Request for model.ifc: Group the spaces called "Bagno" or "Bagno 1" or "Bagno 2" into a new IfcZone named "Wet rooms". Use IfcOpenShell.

First a look at what the model holds.

```python
import ifcopenshell

model = ifcopenshell.open("model.ifc")
print(model.schema)
seen = {}
for space in model.by_type("IfcSpace"):
    seen[space.LongName] = seen.get(space.LongName, 0) + 1
for name, count in sorted(seen.items(), key=str):
    print(count, "x", name)
print("zones:", [z.Name for z in model.by_type("IfcZone")][:20])
```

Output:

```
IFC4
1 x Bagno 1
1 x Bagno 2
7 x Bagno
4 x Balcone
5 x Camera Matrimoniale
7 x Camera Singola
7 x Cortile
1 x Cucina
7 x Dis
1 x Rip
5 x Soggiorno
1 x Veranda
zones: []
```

```python
import ifcopenshell
import ifcopenshell.api.group
import ifcopenshell.api.root

model = ifcopenshell.open("model.ifc")

names = {"Bagno", "Bagno 1", "Bagno 2"}
spaces = [s for s in model.by_type("IfcSpace") if s.LongName in names]

zone = ifcopenshell.api.root.create_entity(model, ifc_class="IfcZone", name="Wet rooms")
ifcopenshell.api.group.assign_group(model, products=spaces, group=zone)
print(len(spaces), "spaces in", zone.Name)

model.write("model_rev.ifc")
```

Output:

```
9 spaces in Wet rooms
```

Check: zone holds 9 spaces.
